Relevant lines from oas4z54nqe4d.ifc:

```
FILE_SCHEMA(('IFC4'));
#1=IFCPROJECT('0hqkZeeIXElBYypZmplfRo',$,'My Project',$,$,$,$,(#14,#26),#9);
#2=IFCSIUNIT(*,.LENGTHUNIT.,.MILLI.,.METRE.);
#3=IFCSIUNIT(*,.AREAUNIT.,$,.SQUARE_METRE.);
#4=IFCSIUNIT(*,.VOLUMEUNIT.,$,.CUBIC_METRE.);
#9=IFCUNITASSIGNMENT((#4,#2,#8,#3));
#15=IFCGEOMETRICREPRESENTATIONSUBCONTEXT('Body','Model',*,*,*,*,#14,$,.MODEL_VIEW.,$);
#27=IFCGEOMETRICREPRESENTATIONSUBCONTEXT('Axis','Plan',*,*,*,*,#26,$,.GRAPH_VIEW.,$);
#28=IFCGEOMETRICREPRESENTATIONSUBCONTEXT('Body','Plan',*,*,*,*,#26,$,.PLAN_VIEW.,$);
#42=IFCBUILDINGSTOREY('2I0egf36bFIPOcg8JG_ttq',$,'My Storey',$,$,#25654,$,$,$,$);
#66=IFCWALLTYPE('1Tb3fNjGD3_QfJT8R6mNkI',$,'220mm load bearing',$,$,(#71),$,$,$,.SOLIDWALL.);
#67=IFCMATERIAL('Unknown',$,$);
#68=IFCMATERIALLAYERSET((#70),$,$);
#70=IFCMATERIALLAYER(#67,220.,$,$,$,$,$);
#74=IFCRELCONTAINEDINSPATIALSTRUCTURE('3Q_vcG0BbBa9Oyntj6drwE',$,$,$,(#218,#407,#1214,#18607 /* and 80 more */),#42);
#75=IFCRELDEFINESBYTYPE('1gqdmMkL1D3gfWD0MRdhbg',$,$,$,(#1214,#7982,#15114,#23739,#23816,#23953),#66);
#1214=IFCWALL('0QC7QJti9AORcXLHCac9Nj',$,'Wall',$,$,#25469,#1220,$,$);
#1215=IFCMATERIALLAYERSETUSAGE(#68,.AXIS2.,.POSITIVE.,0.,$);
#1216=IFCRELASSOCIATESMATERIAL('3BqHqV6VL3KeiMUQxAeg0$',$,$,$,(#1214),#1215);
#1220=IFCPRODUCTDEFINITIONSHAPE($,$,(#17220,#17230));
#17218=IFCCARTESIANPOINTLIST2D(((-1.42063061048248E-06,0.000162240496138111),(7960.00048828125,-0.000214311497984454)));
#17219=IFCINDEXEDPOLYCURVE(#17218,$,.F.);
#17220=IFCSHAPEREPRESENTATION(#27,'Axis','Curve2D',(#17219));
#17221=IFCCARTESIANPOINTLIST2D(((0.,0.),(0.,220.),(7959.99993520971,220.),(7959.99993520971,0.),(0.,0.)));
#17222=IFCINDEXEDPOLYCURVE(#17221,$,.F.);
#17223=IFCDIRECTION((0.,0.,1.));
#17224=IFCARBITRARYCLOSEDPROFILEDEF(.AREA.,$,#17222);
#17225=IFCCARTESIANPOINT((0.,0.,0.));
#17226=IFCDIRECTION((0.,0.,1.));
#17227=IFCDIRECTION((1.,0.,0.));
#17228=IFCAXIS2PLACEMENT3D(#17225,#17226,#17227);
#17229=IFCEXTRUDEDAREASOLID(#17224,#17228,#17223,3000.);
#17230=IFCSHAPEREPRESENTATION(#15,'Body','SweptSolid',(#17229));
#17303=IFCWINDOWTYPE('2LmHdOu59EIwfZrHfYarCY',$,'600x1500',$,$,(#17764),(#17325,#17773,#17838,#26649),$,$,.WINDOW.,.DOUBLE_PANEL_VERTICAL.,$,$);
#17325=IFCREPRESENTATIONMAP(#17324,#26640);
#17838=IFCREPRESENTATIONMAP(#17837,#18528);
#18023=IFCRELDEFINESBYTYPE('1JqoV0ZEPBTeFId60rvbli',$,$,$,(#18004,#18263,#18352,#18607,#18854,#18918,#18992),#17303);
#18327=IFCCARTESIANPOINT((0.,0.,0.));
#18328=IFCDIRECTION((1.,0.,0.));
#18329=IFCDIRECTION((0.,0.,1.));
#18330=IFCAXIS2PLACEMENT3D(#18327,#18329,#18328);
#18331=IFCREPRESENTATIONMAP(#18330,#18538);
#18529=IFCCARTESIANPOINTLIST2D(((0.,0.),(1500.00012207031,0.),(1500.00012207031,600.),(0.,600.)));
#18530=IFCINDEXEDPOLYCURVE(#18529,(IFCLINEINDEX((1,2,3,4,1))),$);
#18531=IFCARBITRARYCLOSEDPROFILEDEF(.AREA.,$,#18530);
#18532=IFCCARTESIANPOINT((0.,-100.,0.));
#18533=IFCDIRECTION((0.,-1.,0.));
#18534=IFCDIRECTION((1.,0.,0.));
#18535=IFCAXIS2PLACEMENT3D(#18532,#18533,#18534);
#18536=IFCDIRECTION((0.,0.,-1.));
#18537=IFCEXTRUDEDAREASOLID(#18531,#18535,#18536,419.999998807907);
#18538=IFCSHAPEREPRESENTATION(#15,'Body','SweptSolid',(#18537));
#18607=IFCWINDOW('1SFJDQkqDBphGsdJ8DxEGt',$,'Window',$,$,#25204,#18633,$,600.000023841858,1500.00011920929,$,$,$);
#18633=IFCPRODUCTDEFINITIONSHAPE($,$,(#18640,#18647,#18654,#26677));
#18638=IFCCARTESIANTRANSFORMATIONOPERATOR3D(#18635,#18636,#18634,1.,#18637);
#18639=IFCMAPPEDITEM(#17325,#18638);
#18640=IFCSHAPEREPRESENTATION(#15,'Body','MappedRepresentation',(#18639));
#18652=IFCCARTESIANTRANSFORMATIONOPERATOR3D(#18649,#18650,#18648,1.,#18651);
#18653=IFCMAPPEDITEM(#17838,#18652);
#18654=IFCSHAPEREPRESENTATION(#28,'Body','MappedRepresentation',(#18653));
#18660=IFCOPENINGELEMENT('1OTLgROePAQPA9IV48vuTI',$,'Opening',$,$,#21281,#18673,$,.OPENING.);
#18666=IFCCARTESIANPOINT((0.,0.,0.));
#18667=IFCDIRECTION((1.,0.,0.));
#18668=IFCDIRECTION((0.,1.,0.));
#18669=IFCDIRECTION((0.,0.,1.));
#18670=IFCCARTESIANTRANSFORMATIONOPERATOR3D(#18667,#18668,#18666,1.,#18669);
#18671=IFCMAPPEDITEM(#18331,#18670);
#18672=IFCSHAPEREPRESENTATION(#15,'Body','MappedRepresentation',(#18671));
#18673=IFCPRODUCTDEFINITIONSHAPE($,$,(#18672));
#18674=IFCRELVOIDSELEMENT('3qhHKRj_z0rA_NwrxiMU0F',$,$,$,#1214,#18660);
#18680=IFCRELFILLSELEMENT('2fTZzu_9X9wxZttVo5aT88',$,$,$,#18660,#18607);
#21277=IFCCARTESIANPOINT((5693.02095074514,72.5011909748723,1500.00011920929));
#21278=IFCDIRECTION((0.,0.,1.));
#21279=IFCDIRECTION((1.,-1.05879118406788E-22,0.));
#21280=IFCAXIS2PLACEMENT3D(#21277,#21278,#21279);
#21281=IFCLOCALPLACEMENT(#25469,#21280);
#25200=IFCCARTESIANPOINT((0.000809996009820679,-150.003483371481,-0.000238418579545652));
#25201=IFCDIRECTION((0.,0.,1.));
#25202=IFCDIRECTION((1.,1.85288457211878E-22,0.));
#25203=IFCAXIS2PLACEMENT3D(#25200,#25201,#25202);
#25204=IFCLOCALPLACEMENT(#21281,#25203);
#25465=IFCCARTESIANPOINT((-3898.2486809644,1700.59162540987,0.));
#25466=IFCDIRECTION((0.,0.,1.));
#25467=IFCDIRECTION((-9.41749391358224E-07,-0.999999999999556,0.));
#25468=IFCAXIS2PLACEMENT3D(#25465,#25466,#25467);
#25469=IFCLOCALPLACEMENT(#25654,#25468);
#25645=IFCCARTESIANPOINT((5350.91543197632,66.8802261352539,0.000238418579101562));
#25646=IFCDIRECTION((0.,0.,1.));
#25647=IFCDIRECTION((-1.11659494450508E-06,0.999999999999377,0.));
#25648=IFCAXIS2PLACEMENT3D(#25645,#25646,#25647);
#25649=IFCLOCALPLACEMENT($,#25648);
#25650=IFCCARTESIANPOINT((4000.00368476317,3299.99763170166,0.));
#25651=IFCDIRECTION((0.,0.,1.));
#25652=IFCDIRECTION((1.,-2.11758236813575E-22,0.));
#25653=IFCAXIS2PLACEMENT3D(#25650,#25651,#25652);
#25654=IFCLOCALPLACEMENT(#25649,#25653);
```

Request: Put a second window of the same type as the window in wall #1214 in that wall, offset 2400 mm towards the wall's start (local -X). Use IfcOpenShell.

```python
import ifcopenshell
import ifcopenshell.api.feature
import ifcopenshell.api.geometry
import ifcopenshell.api.root
import ifcopenshell.geom
import ifcopenshell.util.element
import ifcopenshell.util.placement
import ifcopenshell.util.shape

model = ifcopenshell.open("oas4z54nqe4d.ifc")
settings = ifcopenshell.geom.settings()


def volume(element):
    """Net volume in cubic metres, openings subtracted."""
    shape = ifcopenshell.geom.create_shape(settings, element)
    return ifcopenshell.util.shape.get_volume(shape.geometry)


window = model.by_guid("1SFJDQkqDBphGsdJ8DxEGt")
opening = window.FillsVoids[0].RelatingOpeningElement
wall = opening.VoidsElements[0].RelatingBuildingElement
before = volume(wall)
shift = ifcopenshell.util.placement.get_local_placement(wall.ObjectPlacement)[:3, 0] * -2400.0

# copy_class copies the void relationship, type, container and properties, but no geometry.
new_opening = ifcopenshell.api.root.copy_class(model, product=opening)
new_opening.Representation = ifcopenshell.util.element.copy_deep(
    model, opening.Representation, exclude=["IfcGeometricRepresentationContext", "IfcRepresentationMap"]
)
new_window = ifcopenshell.api.root.copy_class(model, product=window)
new_window.Representation = ifcopenshell.util.element.copy_deep(
    model, window.Representation, exclude=["IfcGeometricRepresentationContext", "IfcRepresentationMap"]
)
ifcopenshell.api.feature.add_filling(model, opening=new_opening, element=new_window)

for old, new in ((opening, new_opening), (window, new_window)):
    matrix = ifcopenshell.util.placement.get_local_placement(old.ObjectPlacement)
    matrix[:3, 3] += shift
    ifcopenshell.api.geometry.edit_object_placement(model, product=new, matrix=matrix, is_si=False)

after = volume(wall)

print(f"wall volume {before:.3f} -> {after:.3f} m3")

model.write("oas4z54nqe4d-out.ifc")
```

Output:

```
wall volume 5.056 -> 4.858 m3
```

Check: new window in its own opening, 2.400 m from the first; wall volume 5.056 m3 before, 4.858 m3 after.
